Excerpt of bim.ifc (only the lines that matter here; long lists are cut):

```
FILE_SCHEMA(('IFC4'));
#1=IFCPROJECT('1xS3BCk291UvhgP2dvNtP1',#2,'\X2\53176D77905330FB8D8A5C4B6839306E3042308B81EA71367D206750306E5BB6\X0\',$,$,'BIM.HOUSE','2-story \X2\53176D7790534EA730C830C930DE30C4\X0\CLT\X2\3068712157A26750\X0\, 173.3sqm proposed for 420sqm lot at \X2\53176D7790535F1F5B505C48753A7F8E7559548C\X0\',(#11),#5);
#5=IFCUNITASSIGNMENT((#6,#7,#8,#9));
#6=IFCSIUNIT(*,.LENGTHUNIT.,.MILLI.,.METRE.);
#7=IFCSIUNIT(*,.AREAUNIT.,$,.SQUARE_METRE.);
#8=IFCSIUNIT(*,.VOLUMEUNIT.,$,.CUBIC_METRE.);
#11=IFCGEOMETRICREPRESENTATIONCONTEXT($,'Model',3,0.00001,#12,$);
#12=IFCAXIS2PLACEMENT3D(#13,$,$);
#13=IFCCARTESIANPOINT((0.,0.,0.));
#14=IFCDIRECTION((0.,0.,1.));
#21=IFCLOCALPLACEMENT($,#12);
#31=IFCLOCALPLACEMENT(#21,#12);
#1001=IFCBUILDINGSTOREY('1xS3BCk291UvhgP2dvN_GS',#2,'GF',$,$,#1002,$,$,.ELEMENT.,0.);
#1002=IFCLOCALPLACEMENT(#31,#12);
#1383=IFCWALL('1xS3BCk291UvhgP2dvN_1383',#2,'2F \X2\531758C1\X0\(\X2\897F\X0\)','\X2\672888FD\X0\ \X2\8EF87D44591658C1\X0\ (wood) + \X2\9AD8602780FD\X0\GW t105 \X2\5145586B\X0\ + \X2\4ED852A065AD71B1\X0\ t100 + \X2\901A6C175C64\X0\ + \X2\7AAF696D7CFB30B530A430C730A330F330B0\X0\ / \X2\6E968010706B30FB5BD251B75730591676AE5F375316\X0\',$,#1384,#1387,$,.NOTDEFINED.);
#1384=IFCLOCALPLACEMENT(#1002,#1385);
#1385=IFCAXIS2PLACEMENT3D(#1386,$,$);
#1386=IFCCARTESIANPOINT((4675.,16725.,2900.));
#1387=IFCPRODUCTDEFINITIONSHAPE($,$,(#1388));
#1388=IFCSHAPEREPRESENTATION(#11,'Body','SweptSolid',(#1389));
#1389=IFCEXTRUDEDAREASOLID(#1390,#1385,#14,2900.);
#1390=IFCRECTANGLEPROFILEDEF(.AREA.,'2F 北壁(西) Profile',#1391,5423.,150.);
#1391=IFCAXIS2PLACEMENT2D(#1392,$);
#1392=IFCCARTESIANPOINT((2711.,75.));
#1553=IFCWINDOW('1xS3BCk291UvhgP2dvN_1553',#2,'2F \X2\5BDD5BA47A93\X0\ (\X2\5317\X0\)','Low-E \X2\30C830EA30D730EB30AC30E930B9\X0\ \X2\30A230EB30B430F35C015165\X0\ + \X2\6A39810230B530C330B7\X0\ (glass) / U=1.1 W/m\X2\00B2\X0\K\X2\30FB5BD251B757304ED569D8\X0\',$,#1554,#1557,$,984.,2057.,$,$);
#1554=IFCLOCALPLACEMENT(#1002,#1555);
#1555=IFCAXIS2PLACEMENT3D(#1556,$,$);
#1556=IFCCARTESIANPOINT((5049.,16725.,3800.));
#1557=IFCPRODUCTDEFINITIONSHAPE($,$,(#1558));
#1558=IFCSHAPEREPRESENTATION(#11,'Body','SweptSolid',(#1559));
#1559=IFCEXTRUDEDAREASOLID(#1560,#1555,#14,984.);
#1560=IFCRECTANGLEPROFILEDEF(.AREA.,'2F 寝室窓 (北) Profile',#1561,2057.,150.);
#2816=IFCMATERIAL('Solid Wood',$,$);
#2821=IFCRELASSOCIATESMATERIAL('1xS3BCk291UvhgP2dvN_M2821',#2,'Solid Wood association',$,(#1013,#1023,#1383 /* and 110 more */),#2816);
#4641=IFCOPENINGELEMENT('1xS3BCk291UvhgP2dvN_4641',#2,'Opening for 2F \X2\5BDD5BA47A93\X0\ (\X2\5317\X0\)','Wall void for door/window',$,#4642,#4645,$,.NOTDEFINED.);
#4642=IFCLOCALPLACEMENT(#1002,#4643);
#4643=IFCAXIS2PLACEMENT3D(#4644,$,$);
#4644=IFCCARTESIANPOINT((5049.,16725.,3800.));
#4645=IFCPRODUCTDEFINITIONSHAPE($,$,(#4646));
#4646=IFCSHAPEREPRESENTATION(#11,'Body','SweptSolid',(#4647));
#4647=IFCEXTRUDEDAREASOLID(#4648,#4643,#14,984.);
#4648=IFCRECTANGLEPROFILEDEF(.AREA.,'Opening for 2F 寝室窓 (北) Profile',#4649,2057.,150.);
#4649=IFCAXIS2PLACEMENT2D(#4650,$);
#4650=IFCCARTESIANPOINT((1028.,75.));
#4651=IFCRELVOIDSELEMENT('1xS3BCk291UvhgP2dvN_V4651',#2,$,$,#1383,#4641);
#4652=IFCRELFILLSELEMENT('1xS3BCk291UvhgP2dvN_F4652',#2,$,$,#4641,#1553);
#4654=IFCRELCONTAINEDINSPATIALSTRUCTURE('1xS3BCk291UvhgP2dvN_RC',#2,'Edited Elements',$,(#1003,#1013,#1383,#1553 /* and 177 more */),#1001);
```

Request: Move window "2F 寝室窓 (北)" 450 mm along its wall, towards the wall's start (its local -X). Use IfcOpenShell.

```python
import ifcopenshell
import ifcopenshell.api.geometry
import ifcopenshell.util.placement
import ifcopenshell.util.unit

model = ifcopenshell.open("bim.ifc")
unit_scale = ifcopenshell.util.unit.calculate_unit_scale(model)

window = model.by_id(1553)
opening = window.FillsVoids[0].RelatingOpeningElement
wall = opening.VoidsElements[0].RelatingBuildingElement

wall_matrix = ifcopenshell.util.placement.get_local_placement(wall.ObjectPlacement)
shift = wall_matrix[:3, 0] * -0.45 / unit_scale
before = ifcopenshell.util.placement.get_local_placement(window.ObjectPlacement)[:3, 3].copy()

# The window is not placed relative to its opening, so move both.
for product in (opening, window):
    matrix = ifcopenshell.util.placement.get_local_placement(product.ObjectPlacement)
    matrix[:3, 3] += shift
    ifcopenshell.api.geometry.edit_object_placement(model, product=product, matrix=matrix, is_si=False)

after = ifcopenshell.util.placement.get_local_placement(window.ObjectPlacement)[:3, 3]
print("window moved by", (after - before).round(3) + 0.0)

model.write("bim-out.ifc")
```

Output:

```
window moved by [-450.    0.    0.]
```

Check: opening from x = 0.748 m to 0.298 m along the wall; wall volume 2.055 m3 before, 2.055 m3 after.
